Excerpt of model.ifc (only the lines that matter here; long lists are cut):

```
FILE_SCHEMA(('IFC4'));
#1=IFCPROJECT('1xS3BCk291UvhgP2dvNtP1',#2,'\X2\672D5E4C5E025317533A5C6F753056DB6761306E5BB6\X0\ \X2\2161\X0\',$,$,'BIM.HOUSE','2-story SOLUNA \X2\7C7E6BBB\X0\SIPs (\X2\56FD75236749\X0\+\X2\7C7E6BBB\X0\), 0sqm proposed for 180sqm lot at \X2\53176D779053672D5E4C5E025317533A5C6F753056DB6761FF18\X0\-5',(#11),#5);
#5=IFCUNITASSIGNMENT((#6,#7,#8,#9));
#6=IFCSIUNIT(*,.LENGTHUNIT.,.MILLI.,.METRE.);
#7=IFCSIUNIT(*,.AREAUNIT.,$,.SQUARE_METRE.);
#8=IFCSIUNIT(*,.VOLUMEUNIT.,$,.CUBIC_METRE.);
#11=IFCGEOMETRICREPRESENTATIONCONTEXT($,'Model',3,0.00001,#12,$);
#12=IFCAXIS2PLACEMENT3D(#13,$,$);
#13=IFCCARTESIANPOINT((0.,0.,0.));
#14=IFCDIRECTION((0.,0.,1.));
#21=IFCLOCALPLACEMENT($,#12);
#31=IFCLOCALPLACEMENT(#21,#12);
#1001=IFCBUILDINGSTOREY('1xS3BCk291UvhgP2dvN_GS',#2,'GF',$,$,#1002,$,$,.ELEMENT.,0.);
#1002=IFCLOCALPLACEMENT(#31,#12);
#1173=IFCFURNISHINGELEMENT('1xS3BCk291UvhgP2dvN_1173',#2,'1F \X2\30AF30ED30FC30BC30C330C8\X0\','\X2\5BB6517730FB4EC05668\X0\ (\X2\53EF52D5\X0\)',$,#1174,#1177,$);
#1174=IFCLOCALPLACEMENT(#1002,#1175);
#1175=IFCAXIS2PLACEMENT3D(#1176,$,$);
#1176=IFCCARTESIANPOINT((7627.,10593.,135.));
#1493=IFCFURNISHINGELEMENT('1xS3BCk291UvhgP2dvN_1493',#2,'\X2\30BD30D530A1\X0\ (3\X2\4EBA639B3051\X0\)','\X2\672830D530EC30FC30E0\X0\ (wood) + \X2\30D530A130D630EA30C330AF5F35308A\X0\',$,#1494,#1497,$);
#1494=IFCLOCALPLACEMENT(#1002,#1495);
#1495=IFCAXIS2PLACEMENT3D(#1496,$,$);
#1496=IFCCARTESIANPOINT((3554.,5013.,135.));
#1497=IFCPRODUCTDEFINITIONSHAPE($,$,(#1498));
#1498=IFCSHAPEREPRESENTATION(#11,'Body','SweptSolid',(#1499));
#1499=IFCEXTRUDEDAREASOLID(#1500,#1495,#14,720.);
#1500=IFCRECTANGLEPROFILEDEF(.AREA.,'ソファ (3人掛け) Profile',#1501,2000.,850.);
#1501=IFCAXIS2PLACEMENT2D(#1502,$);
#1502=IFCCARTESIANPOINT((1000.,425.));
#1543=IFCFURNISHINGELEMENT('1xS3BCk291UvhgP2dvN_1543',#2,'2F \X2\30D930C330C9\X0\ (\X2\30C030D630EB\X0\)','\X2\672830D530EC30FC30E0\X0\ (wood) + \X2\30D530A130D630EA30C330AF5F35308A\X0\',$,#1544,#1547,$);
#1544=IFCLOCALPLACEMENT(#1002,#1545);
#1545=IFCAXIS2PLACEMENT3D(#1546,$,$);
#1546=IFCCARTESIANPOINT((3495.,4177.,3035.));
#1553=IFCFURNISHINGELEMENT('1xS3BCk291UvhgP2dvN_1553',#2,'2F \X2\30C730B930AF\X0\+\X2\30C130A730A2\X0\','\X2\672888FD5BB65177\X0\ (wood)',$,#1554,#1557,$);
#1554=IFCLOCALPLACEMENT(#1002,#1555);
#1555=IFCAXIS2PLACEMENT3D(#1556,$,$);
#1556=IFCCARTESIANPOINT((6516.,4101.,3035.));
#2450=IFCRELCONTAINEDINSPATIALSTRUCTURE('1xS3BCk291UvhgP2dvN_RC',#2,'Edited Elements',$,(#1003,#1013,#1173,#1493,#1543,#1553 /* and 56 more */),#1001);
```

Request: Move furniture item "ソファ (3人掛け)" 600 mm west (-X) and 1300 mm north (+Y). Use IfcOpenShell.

```python
import ifcopenshell
import ifcopenshell.api.geometry
import ifcopenshell.util.placement
import ifcopenshell.util.unit

model = ifcopenshell.open("model.ifc")
unit_scale = ifcopenshell.util.unit.calculate_unit_scale(model)

item = model.by_guid("1xS3BCk291UvhgP2dvN_1493")
matrix = ifcopenshell.util.placement.get_local_placement(item.ObjectPlacement)
matrix[0, 3] -= 0.6 / unit_scale
matrix[1, 3] += 1.3 / unit_scale
ifcopenshell.api.geometry.edit_object_placement(model, product=item, matrix=matrix, is_si=False)

print(ifcopenshell.util.placement.get_local_placement(item.ObjectPlacement).round(3) + 0.0)

model.write("model_rev.ifc")
```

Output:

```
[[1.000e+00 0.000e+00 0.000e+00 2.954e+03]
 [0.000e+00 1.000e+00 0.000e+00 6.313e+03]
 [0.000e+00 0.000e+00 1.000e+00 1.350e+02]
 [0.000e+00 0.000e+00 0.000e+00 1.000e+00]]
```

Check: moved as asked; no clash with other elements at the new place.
